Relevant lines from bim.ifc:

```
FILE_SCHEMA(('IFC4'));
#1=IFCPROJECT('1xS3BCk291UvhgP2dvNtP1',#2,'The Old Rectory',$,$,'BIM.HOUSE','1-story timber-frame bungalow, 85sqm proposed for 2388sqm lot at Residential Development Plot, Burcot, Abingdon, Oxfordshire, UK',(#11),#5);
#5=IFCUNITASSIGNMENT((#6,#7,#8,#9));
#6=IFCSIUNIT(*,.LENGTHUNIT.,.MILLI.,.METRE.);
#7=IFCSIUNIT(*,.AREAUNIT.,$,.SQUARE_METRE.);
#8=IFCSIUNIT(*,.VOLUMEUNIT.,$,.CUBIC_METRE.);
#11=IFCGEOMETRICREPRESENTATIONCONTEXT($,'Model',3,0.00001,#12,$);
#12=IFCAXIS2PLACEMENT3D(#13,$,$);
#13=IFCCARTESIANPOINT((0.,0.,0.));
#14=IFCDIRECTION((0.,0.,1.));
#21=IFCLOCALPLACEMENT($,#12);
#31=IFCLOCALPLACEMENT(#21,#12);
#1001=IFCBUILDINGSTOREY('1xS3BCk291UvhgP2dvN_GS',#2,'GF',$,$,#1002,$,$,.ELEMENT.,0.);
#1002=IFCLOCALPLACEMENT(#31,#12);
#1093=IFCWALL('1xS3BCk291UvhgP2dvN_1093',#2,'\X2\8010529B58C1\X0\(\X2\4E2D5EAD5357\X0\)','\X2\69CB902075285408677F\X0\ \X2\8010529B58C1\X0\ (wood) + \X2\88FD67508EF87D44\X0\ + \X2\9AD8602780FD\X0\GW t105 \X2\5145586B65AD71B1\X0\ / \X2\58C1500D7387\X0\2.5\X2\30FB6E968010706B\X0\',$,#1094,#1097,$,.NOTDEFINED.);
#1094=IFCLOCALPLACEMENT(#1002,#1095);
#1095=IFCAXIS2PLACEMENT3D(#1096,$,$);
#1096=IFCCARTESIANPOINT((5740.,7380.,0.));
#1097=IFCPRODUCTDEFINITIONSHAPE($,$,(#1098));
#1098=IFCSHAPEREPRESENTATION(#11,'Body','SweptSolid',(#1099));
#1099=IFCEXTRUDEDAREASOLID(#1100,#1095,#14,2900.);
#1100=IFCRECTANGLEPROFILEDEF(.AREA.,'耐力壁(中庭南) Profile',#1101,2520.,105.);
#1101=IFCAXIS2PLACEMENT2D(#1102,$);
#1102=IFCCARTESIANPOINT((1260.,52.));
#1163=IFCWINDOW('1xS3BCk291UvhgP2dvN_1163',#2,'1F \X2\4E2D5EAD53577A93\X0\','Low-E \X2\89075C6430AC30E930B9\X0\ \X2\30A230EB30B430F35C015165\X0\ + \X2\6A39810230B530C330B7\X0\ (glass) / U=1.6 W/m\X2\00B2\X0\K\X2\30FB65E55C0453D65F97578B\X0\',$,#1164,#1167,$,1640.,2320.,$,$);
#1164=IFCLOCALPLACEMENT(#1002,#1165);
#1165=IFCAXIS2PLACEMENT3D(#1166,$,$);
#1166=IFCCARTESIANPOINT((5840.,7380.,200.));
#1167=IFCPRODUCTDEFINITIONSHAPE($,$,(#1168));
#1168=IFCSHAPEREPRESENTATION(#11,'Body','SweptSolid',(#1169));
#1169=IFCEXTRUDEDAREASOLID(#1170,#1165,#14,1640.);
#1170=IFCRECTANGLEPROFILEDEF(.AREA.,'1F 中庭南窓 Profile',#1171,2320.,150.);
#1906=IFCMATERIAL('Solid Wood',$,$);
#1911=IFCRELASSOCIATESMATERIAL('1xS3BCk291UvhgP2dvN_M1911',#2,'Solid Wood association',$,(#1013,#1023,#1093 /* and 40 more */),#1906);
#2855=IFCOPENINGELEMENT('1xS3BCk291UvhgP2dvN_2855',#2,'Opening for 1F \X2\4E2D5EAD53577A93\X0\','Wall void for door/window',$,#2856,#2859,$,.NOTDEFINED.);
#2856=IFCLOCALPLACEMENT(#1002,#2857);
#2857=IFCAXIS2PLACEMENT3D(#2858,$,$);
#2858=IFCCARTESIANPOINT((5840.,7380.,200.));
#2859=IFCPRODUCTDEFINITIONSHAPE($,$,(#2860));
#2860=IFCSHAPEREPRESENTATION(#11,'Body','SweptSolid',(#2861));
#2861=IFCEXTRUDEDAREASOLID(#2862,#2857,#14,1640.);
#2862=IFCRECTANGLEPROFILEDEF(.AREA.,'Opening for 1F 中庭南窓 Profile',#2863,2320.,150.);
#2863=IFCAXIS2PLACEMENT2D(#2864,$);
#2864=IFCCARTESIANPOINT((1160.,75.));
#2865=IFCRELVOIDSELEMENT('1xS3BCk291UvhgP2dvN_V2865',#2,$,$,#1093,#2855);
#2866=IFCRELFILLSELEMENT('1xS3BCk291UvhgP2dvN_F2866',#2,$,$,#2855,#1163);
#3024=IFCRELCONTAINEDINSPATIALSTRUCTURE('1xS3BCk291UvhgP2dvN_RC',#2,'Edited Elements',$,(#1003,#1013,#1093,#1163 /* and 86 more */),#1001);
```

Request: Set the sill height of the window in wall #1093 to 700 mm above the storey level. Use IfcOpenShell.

```python
import numpy as np
import ifcopenshell
import ifcopenshell.api.geometry
import ifcopenshell.geom
import ifcopenshell.util.element
import ifcopenshell.util.placement
import ifcopenshell.util.shape
import ifcopenshell.util.unit

model = ifcopenshell.open("bim.ifc")
unit_scale = ifcopenshell.util.unit.calculate_unit_scale(model)

window = model.by_guid("1xS3BCk291UvhgP2dvN_1163")
opening = window.FillsVoids[0].RelatingOpeningElement
storey = ifcopenshell.util.element.get_container(window, ifc_class="IfcBuildingStorey")
level = ifcopenshell.util.placement.get_local_placement(storey.ObjectPlacement)[2, 3]

# The opening's origin need not be at the sill, so measure its lowest point.
shape = ifcopenshell.geom.create_shape(ifcopenshell.geom.settings(), opening)
bottom = ifcopenshell.util.shape.get_shape_bottom_elevation(shape, shape.geometry) / unit_scale
dz = level + 0.7 / unit_scale - bottom

shift = np.array([0.0, 0.0, dz])
# The window is not placed relative to its opening, so move both.
for product in (opening, window):
    matrix = ifcopenshell.util.placement.get_local_placement(product.ObjectPlacement)
    matrix[:3, 3] += shift
    ifcopenshell.api.geometry.edit_object_placement(model, product=product, matrix=matrix, is_si=False)

print(f"moved by {dz * unit_scale:+.3f} m")

model.write("bim_v2.ifc")
```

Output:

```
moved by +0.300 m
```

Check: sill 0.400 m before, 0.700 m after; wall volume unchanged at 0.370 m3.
